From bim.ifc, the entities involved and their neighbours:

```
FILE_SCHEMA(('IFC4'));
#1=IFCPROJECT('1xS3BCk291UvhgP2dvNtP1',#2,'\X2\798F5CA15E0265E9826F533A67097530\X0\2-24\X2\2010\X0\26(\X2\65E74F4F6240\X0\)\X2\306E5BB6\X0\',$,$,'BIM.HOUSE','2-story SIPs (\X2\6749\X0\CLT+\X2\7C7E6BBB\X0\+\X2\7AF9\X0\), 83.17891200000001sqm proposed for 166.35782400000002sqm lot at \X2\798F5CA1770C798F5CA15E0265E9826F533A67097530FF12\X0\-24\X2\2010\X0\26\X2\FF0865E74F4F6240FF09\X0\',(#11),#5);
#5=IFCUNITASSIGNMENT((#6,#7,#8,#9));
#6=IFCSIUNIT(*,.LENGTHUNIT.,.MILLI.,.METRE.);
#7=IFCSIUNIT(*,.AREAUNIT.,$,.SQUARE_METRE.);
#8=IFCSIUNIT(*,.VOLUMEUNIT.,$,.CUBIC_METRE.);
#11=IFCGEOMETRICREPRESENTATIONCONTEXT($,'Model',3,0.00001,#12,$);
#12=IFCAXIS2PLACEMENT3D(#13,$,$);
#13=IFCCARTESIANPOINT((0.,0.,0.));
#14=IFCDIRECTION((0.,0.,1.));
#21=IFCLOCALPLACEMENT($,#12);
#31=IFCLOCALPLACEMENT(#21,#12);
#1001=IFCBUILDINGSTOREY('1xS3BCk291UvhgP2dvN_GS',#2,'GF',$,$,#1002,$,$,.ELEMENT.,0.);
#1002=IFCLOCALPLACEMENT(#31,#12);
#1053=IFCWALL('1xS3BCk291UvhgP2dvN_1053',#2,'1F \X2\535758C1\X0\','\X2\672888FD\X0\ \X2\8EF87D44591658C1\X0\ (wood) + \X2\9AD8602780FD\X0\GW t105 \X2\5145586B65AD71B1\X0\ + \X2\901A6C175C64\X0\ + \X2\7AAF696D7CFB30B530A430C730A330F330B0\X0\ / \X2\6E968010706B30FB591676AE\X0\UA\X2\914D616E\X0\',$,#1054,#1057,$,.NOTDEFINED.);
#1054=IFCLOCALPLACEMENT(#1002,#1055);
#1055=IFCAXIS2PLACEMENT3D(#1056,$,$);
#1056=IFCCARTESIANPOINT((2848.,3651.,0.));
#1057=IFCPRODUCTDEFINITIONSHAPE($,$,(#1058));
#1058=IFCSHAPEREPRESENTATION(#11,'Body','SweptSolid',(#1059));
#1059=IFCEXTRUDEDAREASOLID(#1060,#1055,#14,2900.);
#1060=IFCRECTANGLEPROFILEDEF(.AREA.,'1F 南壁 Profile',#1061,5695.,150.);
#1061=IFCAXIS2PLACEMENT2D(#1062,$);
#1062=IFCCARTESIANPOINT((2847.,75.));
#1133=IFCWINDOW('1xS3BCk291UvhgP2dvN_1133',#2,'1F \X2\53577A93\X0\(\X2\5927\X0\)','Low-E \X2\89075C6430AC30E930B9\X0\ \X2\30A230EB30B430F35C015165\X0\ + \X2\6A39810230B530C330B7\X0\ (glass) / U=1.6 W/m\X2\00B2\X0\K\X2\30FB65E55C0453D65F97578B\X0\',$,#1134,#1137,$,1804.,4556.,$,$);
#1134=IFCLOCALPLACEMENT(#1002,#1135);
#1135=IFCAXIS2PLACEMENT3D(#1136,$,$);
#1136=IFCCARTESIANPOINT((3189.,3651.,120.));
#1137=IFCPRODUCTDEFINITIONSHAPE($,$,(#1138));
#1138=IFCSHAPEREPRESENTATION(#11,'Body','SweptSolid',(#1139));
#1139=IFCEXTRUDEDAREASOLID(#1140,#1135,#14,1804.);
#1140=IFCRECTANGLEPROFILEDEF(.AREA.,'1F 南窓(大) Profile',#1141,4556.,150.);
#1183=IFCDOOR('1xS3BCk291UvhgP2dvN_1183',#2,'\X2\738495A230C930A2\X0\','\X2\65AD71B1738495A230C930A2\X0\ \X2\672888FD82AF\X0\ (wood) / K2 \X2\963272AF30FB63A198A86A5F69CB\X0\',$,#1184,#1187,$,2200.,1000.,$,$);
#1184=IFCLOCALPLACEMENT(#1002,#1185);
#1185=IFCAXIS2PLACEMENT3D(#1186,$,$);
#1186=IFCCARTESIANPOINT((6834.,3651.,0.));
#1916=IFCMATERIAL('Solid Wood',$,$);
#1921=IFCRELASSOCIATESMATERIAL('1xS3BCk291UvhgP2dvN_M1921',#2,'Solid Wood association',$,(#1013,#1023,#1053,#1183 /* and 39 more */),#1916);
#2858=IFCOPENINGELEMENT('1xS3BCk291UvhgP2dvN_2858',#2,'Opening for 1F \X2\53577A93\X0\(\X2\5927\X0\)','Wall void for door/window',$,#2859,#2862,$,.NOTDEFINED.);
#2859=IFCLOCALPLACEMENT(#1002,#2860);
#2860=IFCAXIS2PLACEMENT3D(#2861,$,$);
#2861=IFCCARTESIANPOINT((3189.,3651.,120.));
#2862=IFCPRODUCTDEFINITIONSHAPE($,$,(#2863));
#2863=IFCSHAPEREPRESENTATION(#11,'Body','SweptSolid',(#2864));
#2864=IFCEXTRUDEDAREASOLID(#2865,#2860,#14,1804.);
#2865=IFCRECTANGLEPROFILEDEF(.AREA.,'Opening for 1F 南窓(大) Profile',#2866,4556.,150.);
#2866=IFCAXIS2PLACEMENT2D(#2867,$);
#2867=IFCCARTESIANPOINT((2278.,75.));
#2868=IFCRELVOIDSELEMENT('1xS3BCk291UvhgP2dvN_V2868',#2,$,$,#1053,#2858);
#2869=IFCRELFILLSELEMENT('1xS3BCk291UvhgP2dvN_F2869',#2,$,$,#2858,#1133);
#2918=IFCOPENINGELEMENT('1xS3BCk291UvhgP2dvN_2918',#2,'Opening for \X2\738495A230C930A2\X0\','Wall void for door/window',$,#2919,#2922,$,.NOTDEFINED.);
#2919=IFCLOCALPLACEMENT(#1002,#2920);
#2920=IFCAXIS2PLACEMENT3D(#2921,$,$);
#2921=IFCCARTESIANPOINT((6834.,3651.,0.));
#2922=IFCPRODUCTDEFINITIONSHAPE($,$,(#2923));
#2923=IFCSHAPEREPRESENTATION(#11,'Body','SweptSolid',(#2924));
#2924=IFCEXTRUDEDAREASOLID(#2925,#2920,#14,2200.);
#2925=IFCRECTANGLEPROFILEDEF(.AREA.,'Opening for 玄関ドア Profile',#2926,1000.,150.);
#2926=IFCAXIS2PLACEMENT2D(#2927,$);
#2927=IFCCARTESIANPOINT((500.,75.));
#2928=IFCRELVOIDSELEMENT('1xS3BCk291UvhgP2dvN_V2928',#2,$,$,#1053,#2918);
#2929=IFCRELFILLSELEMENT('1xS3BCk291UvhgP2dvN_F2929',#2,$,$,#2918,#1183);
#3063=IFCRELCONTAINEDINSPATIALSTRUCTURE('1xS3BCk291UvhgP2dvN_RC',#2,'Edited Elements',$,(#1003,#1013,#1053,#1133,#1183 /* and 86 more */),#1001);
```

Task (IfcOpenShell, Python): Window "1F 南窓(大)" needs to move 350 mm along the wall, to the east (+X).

```python
import ifcopenshell
import ifcopenshell.api.geometry
import ifcopenshell.util.placement
import ifcopenshell.util.unit

model = ifcopenshell.open("bim.ifc")
unit_scale = ifcopenshell.util.unit.calculate_unit_scale(model)

window = model.by_guid("1xS3BCk291UvhgP2dvN_1133")
opening = window.FillsVoids[0].RelatingOpeningElement
wall = opening.VoidsElements[0].RelatingBuildingElement

wall_matrix = ifcopenshell.util.placement.get_local_placement(wall.ObjectPlacement)
shift = wall_matrix[:3, 0] * 0.35 / unit_scale
before = ifcopenshell.util.placement.get_local_placement(window.ObjectPlacement)[:3, 3].copy()

# The window is not placed relative to its opening, so move both.
for product in (opening, window):
    matrix = ifcopenshell.util.placement.get_local_placement(product.ObjectPlacement)
    matrix[:3, 3] += shift
    ifcopenshell.api.geometry.edit_object_placement(model, product=product, matrix=matrix, is_si=False)

after = ifcopenshell.util.placement.get_local_placement(window.ObjectPlacement)[:3, 3]
print("window moved by", (after - before).round(3) + 0.0)

model.write("bim_updated.ifc")
```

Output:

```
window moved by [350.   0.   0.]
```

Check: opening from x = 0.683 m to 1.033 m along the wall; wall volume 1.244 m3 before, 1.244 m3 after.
